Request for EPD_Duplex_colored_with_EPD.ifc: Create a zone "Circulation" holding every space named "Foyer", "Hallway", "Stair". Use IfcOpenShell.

First a look at what the model holds.

```python
import ifcopenshell

model = ifcopenshell.open("EPD_Duplex_colored_with_EPD.ifc")
print(model.schema)
seen = {}
for space in model.by_type("IfcSpace"):
    seen[space.LongName] = seen.get(space.LongName, 0) + 1
for name, count in sorted(seen.items(), key=str):
    print(count, "x", name)
print("zones:", [z.Name for z in model.by_type("IfcZone")][:20])
```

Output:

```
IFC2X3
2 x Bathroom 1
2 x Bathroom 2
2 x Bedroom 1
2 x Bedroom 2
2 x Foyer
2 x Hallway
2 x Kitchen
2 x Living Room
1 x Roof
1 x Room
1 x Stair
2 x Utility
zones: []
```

```python
import ifcopenshell
import ifcopenshell.api.group
import ifcopenshell.api.root

model = ifcopenshell.open("EPD_Duplex_colored_with_EPD.ifc")

names = {"Foyer", "Hallway", "Stair"}
spaces = [s for s in model.by_type("IfcSpace") if s.LongName in names]

zone = ifcopenshell.api.root.create_entity(model, ifc_class="IfcZone", name="Circulation")
ifcopenshell.api.group.assign_group(model, products=spaces, group=zone)
print(len(spaces), "spaces in", zone.Name)

model.write("EPD_Duplex_colored_with_EPD-out.ifc")
```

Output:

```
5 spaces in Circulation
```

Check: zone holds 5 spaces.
